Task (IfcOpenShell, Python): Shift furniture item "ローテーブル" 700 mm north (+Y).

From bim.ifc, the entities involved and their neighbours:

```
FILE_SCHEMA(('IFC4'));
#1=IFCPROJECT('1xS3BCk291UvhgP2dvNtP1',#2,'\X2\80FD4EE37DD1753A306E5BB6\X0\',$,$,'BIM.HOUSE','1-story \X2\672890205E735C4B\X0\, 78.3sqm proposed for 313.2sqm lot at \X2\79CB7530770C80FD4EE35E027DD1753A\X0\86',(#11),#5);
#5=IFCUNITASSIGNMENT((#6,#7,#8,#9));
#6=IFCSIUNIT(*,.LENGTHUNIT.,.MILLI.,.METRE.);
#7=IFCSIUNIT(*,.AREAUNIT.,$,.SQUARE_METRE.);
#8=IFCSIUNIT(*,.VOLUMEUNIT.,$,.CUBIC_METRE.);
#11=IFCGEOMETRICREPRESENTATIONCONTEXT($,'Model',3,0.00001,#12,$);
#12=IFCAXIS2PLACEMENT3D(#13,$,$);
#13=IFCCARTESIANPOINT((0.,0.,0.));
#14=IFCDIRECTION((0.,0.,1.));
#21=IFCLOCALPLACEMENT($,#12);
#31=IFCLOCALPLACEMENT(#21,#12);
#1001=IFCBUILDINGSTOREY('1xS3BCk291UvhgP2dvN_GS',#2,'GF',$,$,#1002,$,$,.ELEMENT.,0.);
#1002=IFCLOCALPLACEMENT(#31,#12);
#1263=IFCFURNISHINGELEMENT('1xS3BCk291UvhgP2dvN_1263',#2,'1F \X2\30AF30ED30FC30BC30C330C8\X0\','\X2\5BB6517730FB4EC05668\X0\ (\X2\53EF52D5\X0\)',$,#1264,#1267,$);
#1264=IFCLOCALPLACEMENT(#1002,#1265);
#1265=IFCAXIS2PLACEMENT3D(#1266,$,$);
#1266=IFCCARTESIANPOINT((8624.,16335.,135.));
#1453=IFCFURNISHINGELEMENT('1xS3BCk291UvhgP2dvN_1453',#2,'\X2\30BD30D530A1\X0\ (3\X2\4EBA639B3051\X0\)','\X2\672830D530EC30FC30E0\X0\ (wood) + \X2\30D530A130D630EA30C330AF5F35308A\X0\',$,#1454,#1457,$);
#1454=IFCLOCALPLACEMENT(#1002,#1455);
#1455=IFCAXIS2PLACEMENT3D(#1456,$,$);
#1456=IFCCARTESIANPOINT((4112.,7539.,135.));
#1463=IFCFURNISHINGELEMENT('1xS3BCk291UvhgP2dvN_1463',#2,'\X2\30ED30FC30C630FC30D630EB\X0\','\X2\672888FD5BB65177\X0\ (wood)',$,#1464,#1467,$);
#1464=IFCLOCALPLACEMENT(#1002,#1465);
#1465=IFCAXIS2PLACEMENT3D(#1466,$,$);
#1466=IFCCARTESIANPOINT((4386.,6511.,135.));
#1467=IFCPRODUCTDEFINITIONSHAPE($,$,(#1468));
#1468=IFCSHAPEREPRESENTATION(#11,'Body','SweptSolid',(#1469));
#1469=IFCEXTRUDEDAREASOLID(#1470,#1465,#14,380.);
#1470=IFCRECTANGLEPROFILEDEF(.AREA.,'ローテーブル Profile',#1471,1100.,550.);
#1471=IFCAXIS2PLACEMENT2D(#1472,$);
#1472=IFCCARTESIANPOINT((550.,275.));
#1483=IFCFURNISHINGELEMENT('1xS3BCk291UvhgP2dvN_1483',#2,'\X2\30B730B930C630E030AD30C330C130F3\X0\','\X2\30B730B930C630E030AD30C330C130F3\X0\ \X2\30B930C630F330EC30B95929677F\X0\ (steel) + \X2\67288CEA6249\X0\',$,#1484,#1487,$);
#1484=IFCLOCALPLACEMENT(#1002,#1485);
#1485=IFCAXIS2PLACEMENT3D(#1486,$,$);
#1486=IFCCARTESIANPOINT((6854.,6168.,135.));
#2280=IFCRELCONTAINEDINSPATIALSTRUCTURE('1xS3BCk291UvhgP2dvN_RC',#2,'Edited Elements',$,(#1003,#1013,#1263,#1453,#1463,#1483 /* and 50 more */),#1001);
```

```python
import ifcopenshell
import ifcopenshell.api.geometry
import ifcopenshell.util.placement

model = ifcopenshell.open("bim.ifc")

item = model.by_id(1463)
matrix = ifcopenshell.util.placement.get_local_placement(item.ObjectPlacement)
matrix[1, 3] += 700.0
ifcopenshell.api.geometry.edit_object_placement(model, product=item, matrix=matrix, is_si=False)

print(ifcopenshell.util.placement.get_local_placement(item.ObjectPlacement).round(3) + 0.0)

model.write("bim_updated.ifc")
```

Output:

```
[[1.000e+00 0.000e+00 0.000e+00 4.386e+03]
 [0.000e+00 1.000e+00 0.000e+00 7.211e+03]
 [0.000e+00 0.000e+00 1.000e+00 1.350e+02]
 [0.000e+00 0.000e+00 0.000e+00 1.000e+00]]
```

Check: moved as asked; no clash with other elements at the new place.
